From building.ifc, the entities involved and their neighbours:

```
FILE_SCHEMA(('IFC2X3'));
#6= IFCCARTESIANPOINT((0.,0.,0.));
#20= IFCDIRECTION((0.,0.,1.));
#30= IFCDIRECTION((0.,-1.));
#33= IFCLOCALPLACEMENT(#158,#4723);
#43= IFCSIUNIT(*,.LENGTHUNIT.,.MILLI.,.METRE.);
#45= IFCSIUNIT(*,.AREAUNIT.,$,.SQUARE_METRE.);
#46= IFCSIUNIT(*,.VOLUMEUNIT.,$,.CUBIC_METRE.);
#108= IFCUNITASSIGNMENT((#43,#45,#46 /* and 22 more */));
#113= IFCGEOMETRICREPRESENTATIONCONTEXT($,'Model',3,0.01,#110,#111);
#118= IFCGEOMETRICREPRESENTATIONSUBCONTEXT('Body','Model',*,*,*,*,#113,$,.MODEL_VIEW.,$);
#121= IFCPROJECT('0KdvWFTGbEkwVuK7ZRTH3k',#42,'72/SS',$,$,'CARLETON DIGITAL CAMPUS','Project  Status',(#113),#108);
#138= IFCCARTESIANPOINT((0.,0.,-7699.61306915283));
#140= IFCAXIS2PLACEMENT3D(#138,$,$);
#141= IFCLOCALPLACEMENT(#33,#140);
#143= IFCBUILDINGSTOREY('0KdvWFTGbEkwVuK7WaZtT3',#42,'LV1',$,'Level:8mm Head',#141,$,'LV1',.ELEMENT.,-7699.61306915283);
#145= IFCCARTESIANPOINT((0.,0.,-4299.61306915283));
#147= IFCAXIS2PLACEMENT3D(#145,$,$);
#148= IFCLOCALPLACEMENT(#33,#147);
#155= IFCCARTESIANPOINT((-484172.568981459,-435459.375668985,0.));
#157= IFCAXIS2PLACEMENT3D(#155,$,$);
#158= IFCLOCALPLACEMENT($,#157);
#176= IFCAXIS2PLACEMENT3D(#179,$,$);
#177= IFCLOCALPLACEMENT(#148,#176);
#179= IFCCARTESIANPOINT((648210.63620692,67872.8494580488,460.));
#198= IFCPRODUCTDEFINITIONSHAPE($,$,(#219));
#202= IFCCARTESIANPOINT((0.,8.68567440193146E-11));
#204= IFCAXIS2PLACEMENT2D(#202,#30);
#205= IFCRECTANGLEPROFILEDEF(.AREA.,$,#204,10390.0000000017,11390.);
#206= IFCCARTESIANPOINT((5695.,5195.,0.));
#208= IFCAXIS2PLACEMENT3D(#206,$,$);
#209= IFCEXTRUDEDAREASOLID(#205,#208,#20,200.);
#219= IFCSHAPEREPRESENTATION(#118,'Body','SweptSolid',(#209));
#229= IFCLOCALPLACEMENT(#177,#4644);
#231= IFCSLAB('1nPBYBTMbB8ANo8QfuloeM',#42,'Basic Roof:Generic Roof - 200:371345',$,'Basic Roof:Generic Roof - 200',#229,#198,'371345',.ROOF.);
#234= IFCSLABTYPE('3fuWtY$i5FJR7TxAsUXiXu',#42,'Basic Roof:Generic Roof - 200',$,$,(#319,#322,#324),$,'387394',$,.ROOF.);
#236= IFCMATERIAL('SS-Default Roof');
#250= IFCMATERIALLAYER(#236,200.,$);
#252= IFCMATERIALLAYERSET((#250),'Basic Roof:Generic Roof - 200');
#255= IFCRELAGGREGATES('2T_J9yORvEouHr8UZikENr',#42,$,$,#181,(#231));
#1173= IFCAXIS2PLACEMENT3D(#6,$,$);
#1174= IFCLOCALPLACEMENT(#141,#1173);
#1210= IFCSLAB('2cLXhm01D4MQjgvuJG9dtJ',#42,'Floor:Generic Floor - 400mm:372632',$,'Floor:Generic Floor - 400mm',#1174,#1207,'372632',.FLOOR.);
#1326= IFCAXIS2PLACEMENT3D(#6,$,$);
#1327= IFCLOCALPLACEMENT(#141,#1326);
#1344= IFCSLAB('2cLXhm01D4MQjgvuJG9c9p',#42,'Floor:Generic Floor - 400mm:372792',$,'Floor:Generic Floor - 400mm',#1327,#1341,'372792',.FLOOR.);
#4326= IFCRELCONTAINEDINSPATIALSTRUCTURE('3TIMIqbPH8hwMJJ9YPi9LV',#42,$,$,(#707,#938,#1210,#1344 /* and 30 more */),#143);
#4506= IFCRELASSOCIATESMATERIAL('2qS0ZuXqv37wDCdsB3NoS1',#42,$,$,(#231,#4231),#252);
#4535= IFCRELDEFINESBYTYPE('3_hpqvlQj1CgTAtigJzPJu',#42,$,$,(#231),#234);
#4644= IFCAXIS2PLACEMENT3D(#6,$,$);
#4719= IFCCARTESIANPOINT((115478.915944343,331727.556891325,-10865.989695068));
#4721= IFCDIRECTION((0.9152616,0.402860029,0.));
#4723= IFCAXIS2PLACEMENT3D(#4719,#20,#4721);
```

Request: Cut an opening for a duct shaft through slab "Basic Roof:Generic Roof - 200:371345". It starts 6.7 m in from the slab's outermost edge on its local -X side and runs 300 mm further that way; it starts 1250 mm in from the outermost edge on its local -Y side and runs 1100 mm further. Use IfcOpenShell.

```python
import numpy as np
import ifcopenshell
import ifcopenshell.api.feature
import ifcopenshell.api.geometry
import ifcopenshell.api.root
import ifcopenshell.geom
import ifcopenshell.util.placement
import ifcopenshell.util.representation
import ifcopenshell.util.shape
import ifcopenshell.util.unit

model = ifcopenshell.open("building.ifc")
unit_scale = ifcopenshell.util.unit.calculate_unit_scale(model)
settings = ifcopenshell.geom.settings()


def volume(element):
    """Net volume in cubic metres, openings subtracted."""
    shape = ifcopenshell.geom.create_shape(settings, element)
    return ifcopenshell.util.shape.get_volume(shape.geometry)


slab = model.by_guid("1nPBYBTMbB8ANo8QfuloeM")
before = volume(slab)

# Extent in the slab's own axes, in metres. The edges named are its -X and -Y sides.
slab_shape = ifcopenshell.geom.create_shape(settings, slab)
vertices = ifcopenshell.util.shape.get_vertices(slab_shape.geometry)
x_min, y_min, bottom = vertices.min(axis=0)
top = vertices[:, 2].max()

opening = ifcopenshell.api.root.create_entity(model, ifc_class="IfcOpeningElement", name="Duct shaft opening")
context = ifcopenshell.util.representation.get_context(model, "Model", "Body", "MODEL_VIEW")
width, depth = 0.3, 1.1
outline = [(0.0, 0.0), (width, 0.0), (width, depth), (0.0, depth), (0.0, 0.0)]
# Overshoot both faces by 50 mm so the cut is clean.
shape = ifcopenshell.api.geometry.add_slab_representation(
    model, context=context, depth=top - bottom + 0.1, polyline=outline
)
ifcopenshell.api.geometry.assign_representation(model, product=opening, representation=shape)

matrix = ifcopenshell.util.placement.get_local_placement(slab.ObjectPlacement)
matrix[:, 3] = matrix @ np.append(np.array([x_min + 6.7, y_min + 1.25, bottom - 0.05]) / unit_scale, 1.0)
ifcopenshell.api.geometry.edit_object_placement(model, product=opening, matrix=matrix, is_si=False)
ifcopenshell.api.feature.add_feature(model, feature=opening, element=slab)

after = volume(slab)

print(f"slab volume {before:.3f} -> {after:.3f} m3")

model.write("building_updated.ifc")
```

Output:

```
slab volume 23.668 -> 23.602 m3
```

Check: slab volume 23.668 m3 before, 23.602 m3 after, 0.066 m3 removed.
